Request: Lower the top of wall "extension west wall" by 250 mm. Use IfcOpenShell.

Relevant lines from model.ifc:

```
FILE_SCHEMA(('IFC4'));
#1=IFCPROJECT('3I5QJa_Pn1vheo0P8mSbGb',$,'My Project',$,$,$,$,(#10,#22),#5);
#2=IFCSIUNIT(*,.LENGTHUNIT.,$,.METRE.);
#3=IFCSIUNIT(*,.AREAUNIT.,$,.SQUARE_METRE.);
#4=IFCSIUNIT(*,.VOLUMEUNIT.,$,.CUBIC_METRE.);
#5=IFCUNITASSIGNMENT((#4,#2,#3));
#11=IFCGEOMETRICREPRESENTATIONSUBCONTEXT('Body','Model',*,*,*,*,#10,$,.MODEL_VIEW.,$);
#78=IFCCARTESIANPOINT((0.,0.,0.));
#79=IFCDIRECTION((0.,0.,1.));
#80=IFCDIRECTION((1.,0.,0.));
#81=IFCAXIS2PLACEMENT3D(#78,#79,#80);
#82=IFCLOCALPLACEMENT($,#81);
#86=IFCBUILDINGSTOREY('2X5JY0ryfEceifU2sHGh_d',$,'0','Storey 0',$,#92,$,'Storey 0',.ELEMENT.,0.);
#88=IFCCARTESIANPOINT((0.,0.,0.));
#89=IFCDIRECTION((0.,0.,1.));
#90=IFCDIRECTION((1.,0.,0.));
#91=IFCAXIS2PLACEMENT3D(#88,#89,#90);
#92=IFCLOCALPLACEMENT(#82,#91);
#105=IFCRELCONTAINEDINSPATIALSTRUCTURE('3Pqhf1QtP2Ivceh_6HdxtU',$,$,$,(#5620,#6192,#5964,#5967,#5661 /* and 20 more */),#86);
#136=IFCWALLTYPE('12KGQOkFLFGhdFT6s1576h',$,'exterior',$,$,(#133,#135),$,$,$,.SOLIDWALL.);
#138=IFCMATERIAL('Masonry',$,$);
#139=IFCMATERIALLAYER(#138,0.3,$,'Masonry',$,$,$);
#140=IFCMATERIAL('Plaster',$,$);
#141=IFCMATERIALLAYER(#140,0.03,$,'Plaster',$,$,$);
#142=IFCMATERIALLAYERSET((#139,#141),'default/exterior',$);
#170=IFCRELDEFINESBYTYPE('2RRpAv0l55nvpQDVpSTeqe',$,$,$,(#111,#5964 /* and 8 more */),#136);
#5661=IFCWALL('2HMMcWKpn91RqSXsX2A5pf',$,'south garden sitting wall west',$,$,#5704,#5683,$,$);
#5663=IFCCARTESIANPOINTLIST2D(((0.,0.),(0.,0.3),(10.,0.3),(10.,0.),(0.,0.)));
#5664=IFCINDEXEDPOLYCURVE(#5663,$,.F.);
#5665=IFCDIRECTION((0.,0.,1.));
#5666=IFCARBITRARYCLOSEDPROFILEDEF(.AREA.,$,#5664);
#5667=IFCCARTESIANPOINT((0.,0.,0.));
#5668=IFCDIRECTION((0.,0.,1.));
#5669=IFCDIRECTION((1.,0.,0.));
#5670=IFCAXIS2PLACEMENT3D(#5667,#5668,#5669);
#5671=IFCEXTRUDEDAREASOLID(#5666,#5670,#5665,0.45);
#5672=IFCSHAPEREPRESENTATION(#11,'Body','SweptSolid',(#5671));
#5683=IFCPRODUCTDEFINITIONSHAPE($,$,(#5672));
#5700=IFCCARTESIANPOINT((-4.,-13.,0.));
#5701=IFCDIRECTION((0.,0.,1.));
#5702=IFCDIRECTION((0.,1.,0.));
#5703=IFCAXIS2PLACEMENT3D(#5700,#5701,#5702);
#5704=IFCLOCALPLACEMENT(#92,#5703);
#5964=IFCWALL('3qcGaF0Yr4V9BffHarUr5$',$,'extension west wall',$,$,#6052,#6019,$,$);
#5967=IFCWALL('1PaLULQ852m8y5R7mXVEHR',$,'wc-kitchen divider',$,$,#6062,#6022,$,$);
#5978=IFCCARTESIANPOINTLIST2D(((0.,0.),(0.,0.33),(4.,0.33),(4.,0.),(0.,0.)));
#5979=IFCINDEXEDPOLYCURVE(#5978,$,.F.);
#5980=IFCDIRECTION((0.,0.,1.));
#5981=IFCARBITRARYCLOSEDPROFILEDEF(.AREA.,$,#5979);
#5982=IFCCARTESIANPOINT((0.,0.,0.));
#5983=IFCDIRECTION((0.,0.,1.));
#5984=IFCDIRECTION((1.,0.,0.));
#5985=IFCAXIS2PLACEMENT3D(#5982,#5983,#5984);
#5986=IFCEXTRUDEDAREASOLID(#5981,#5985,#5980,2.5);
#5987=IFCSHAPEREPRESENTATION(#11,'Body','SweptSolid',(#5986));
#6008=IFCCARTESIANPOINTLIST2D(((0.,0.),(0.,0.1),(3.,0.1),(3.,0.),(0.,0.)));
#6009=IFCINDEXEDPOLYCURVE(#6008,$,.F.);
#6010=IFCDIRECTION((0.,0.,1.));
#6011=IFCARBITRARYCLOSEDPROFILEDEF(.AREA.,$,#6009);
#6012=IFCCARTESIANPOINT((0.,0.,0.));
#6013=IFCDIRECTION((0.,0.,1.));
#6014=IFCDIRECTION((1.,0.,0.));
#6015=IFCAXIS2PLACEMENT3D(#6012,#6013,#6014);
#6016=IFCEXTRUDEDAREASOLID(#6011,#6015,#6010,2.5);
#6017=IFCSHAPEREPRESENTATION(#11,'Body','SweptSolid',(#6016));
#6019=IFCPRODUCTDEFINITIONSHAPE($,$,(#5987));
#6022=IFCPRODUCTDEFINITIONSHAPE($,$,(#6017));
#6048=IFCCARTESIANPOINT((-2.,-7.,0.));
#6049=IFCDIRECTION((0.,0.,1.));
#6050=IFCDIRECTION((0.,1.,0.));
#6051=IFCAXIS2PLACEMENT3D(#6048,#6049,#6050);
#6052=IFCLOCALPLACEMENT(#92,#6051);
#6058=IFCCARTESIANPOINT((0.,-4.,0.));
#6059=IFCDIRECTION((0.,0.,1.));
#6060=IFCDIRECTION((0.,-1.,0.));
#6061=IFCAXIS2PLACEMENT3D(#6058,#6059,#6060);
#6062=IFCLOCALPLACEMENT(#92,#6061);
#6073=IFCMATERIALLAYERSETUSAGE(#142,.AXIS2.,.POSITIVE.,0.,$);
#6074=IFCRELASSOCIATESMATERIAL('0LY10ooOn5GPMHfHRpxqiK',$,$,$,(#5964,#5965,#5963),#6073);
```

```python
import ifcopenshell
import ifcopenshell.geom
import ifcopenshell.util.representation
import ifcopenshell.util.shape
import ifcopenshell.util.unit

model = ifcopenshell.open("model.ifc")
unit_scale = ifcopenshell.util.unit.calculate_unit_scale(model)
settings = ifcopenshell.geom.settings()


def volume(element):
    """Net volume in cubic metres, openings subtracted."""
    shape = ifcopenshell.geom.create_shape(settings, element)
    return ifcopenshell.util.shape.get_volume(shape.geometry)


wall = model.by_guid("3qcGaF0Yr4V9BffHarUr5$")
before = volume(wall)

body = ifcopenshell.util.representation.get_representation(wall, "Model", "Body")
solid = body.Items[0]
old_height = solid.Depth
solid.Depth -= 0.25 / unit_scale
after = volume(wall)

print(f"height {old_height:g} -> {solid.Depth:g}, volume {before:.3f} -> {after:.3f} m3")

model.write("model_rev.ifc")
```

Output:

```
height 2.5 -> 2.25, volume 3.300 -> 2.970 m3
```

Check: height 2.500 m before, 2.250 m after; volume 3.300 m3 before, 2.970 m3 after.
